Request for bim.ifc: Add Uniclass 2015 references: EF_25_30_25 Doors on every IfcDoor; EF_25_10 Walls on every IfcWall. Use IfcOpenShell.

First a look at what the model holds.

```python
import ifcopenshell

model = ifcopenshell.open("bim.ifc")
print(model.schema)
print("classifications:", [c.Name for c in model.by_type("IfcClassification")])
for ifc_class in ("IfcDoor", "IfcRoof", "IfcStair", "IfcWall", "IfcWindow"):
    print(ifc_class, len(model.by_type(ifc_class)))
```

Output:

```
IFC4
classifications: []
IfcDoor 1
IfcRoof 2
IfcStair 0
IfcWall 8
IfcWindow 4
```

```python
import ifcopenshell
import ifcopenshell.api.classification

model = ifcopenshell.open("bim.ifc")

system = ifcopenshell.api.classification.add_classification(model, classification="Uniclass 2015")

codes = {
    "IfcDoor": ("EF_25_30_25", "Doors"),
    "IfcWall": ("EF_25_10", "Walls"),
}
for ifc_class, (code, name) in codes.items():
    products = model.by_type(ifc_class)
    ifcopenshell.api.classification.add_reference(
        model, products=products, classification=system, identification=code, name=name
    )
    print(code, len(products))

model.write("bim_updated.ifc")
```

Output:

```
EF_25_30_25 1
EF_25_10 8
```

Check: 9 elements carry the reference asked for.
